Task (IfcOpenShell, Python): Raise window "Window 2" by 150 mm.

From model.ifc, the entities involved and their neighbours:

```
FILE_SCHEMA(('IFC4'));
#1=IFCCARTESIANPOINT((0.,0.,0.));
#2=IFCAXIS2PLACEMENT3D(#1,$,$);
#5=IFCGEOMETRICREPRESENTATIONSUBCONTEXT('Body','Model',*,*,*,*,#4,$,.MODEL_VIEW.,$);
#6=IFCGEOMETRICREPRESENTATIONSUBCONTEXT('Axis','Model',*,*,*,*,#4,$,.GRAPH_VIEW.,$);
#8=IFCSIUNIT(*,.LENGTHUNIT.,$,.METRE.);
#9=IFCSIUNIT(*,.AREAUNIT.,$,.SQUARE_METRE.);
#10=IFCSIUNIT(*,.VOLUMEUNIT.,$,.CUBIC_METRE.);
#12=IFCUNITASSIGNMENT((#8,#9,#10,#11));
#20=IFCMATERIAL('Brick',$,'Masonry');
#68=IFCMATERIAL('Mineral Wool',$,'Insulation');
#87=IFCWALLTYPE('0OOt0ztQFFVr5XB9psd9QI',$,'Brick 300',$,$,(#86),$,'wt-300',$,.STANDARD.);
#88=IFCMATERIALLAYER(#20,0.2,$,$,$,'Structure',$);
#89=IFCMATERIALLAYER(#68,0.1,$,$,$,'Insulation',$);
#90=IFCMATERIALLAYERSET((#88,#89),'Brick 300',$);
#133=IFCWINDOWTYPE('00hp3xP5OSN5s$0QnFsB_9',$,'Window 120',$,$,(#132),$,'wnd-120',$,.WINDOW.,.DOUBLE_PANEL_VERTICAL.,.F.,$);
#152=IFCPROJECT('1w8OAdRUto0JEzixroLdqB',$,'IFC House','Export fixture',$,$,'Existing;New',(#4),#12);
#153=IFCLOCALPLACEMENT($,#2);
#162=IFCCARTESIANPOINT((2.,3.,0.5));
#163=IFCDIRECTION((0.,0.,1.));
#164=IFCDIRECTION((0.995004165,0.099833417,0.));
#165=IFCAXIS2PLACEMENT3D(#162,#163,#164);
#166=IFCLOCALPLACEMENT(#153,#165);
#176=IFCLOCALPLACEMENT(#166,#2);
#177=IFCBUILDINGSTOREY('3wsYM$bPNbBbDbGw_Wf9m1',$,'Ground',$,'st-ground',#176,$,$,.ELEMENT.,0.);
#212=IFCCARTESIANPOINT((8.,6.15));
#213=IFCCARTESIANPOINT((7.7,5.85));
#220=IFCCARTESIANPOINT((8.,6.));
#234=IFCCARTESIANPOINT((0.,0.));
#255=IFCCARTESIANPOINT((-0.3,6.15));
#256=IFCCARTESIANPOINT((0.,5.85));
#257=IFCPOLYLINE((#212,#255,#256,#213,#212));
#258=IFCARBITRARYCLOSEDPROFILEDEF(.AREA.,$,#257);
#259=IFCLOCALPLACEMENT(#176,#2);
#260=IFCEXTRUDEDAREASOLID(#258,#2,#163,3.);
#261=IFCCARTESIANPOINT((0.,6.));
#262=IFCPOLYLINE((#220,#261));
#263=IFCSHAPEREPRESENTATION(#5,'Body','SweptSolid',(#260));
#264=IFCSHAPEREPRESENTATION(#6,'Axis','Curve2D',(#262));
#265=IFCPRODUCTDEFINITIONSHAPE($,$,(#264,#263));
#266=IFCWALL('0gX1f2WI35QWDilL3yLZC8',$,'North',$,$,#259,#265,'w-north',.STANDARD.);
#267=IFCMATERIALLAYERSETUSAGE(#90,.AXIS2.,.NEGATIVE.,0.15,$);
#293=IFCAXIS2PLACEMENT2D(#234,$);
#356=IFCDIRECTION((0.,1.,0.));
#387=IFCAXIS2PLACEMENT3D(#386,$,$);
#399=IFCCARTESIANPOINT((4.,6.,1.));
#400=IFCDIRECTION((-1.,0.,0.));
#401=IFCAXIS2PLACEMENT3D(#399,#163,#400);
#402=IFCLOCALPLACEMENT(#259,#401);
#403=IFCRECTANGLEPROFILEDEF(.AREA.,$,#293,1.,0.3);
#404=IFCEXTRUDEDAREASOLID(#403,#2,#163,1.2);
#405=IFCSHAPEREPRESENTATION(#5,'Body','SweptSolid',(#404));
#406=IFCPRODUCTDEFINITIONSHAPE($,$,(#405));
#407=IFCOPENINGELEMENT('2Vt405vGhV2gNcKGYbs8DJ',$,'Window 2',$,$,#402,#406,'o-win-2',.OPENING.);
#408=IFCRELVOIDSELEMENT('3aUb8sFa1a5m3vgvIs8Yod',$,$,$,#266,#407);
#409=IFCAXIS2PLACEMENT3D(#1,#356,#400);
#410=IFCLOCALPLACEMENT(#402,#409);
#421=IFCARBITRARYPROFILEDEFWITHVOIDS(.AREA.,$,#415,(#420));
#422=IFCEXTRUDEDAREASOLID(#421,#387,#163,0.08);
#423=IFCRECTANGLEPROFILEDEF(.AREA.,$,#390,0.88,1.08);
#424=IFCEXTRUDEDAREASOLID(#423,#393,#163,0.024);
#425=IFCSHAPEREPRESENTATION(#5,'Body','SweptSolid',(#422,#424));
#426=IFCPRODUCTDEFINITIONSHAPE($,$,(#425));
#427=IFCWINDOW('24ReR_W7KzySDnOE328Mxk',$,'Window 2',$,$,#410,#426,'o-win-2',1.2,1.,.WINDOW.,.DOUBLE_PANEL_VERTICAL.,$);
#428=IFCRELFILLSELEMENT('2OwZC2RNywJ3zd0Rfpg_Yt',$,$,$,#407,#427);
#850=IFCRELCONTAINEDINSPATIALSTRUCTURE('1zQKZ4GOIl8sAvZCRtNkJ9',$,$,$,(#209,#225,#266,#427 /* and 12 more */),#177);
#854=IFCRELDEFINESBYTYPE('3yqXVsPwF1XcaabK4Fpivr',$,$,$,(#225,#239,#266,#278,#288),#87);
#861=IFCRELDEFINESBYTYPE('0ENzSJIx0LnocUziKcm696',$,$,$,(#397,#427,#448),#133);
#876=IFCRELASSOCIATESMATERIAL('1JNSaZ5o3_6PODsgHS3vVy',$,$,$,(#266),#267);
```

```python
import numpy as np
import ifcopenshell
import ifcopenshell.api.geometry
import ifcopenshell.util.placement
import ifcopenshell.util.unit

model = ifcopenshell.open("model.ifc")
unit_scale = ifcopenshell.util.unit.calculate_unit_scale(model)

window = model.by_id(427)
opening = window.FillsVoids[0].RelatingOpeningElement
dz = 0.15

shift = np.array([0.0, 0.0, dz])
# The window is placed relative to its opening, so it follows when the opening moves.
matrix = ifcopenshell.util.placement.get_local_placement(opening.ObjectPlacement)
matrix[:3, 3] += shift
ifcopenshell.api.geometry.edit_object_placement(
    model, product=opening, matrix=matrix, is_si=False, should_transform_children=True
)

print(f"moved by {dz * unit_scale:+.3f} m")

model.write("model_v2.ifc")
```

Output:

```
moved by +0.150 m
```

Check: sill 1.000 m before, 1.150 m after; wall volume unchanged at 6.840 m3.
